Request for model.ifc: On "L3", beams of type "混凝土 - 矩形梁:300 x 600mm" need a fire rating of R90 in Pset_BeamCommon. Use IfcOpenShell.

First a look at what the model holds.

```python
import ifcopenshell
import ifcopenshell.util.element

model = ifcopenshell.open("model.ifc")
print(model.schema)
storey = next(s for s in model.by_type("IfcBuildingStorey") if s.Name == "L3")
beams = [e for e in ifcopenshell.util.element.get_decomposition(storey) if e.is_a("IfcBeam")]
seen = {}
for e in beams:
    element_type = ifcopenshell.util.element.get_type(e)
    key = (element_type.Name if element_type != e and element_type else None, ifcopenshell.util.element.get_pset(e, "Pset_BeamCommon", "FireRating"))
    seen[key] = seen.get(key, 0) + 1
for (name, value), count in sorted(seen.items(), key=str):
    print(count, "x", name, "|", value)
```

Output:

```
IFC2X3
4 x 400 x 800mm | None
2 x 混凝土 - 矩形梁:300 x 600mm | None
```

```python
import ifcopenshell
import ifcopenshell.api.pset
import ifcopenshell.util.element

model = ifcopenshell.open("model.ifc")

storey = next(s for s in model.by_type("IfcBuildingStorey") if s.Name == "L3")
beams = [e for e in ifcopenshell.util.element.get_decomposition(storey) if e.is_a("IfcBeam")]

count = 0
for e in beams:
    element_type = ifcopenshell.util.element.get_type(e)
    if element_type in (None, e) or element_type.Name != "混凝土 - 矩形梁:300 x 600mm":
        continue
    # add_pset returns the element's existing set when there is one.
    pset = ifcopenshell.api.pset.add_pset(model, product=e, name="Pset_BeamCommon")
    ifcopenshell.api.pset.edit_pset(model, pset=pset, properties={"FireRating": "R90"})
    count += 1

print(count, "beams updated")

model.write("model_updated.ifc")
```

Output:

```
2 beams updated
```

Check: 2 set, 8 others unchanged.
